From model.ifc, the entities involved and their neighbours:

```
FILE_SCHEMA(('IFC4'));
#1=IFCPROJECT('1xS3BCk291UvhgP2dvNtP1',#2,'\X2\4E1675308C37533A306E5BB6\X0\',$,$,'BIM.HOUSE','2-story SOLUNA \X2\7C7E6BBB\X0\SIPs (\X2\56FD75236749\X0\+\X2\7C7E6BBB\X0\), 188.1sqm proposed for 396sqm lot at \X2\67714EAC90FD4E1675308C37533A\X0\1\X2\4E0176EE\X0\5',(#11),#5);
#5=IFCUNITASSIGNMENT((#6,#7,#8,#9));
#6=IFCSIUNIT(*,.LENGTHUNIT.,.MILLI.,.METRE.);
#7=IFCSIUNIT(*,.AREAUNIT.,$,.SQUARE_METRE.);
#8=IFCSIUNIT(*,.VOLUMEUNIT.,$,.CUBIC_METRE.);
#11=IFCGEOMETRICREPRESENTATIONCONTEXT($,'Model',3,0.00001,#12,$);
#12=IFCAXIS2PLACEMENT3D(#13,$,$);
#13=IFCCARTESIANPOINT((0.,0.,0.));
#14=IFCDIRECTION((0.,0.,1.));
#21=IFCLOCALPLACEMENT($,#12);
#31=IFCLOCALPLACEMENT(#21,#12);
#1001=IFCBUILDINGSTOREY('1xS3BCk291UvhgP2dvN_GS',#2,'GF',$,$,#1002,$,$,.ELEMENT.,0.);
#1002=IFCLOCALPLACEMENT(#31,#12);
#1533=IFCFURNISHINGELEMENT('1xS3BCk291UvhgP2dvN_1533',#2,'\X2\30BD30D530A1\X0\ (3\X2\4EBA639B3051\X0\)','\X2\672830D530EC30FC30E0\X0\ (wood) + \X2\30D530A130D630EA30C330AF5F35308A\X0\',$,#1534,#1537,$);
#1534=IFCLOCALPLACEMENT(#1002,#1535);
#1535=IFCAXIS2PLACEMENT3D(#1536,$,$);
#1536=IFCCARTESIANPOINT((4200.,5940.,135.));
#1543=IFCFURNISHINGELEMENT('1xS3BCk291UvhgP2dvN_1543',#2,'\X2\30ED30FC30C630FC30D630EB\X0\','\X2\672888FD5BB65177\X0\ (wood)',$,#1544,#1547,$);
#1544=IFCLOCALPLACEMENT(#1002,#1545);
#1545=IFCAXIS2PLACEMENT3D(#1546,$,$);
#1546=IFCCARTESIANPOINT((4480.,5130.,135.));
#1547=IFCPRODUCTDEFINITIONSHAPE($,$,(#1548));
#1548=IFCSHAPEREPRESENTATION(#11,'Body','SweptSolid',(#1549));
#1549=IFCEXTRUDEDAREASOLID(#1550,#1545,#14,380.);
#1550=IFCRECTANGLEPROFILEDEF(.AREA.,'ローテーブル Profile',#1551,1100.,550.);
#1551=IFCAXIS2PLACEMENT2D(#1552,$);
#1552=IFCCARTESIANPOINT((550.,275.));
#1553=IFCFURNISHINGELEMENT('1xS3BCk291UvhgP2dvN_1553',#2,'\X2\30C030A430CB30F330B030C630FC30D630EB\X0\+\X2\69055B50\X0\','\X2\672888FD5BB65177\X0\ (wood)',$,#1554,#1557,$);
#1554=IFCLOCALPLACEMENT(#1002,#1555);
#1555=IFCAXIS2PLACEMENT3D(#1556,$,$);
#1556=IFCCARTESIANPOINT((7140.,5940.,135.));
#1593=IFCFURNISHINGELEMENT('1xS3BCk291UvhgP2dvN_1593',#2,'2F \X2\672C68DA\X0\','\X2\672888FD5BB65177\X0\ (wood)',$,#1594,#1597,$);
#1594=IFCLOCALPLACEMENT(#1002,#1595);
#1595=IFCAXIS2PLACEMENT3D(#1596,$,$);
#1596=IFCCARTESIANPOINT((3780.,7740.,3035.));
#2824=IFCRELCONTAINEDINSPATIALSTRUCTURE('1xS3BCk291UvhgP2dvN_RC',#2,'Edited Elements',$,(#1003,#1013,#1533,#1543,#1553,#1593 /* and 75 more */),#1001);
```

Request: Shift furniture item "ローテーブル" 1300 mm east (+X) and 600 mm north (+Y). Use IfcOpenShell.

```python
import ifcopenshell
import ifcopenshell.api.geometry
import ifcopenshell.util.placement
import ifcopenshell.util.unit

model = ifcopenshell.open("model.ifc")
unit_scale = ifcopenshell.util.unit.calculate_unit_scale(model)

item = model.by_guid("1xS3BCk291UvhgP2dvN_1543")
matrix = ifcopenshell.util.placement.get_local_placement(item.ObjectPlacement)
matrix[0, 3] += 1.3 / unit_scale
matrix[1, 3] += 0.6 / unit_scale
ifcopenshell.api.geometry.edit_object_placement(model, product=item, matrix=matrix, is_si=False)

print(ifcopenshell.util.placement.get_local_placement(item.ObjectPlacement).round(3) + 0.0)

model.write("model-out.ifc")
```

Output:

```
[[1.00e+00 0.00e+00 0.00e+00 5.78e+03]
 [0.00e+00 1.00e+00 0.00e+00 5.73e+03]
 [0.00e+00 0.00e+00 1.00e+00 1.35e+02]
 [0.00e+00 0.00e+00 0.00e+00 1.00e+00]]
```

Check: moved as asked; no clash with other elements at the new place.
